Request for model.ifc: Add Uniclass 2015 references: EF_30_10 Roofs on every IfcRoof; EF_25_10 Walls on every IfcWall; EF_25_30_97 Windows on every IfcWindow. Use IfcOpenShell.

First a look at what the model holds.

```python
import ifcopenshell

model = ifcopenshell.open("model.ifc")
print(model.schema)
print("classifications:", [c.Name for c in model.by_type("IfcClassification")])
for ifc_class in ("IfcDoor", "IfcRoof", "IfcStair", "IfcWall", "IfcWindow"):
    print(ifc_class, len(model.by_type(ifc_class)))
```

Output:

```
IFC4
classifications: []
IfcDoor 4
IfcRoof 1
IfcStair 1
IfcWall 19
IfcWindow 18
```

```python
import ifcopenshell
import ifcopenshell.api.classification

model = ifcopenshell.open("model.ifc")

system = ifcopenshell.api.classification.add_classification(model, classification="Uniclass 2015")

codes = {
    "IfcRoof": ("EF_30_10", "Roofs"),
    "IfcWall": ("EF_25_10", "Walls"),
    "IfcWindow": ("EF_25_30_97", "Windows"),
}
for ifc_class, (code, name) in codes.items():
    products = model.by_type(ifc_class)
    ifcopenshell.api.classification.add_reference(
        model, products=products, classification=system, identification=code, name=name
    )
    print(code, len(products))

model.write("model_edited.ifc")
```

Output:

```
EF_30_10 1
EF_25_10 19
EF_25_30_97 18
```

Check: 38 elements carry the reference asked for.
